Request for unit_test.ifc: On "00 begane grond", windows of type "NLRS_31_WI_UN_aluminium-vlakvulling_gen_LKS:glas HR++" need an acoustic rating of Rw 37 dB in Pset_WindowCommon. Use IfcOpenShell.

First a look at what the model holds.

```python
import ifcopenshell
import ifcopenshell.util.element

model = ifcopenshell.open("unit_test.ifc")
print(model.schema)
storey = next(s for s in model.by_type("IfcBuildingStorey") if s.Name == "00 begane grond")
windows = [e for e in ifcopenshell.util.element.get_decomposition(storey) if e.is_a("IfcWindow")]
seen = {}
for e in windows:
    element_type = ifcopenshell.util.element.get_type(e)
    key = (element_type.Name if element_type != e and element_type else None, ifcopenshell.util.element.get_pset(e, "Pset_WindowCommon", "AcousticRating"))
    seen[key] = seen.get(key, 0) + 1
for (name, value), count in sorted(seen.items(), key=str):
    print(count, "x", name, "|", value)
```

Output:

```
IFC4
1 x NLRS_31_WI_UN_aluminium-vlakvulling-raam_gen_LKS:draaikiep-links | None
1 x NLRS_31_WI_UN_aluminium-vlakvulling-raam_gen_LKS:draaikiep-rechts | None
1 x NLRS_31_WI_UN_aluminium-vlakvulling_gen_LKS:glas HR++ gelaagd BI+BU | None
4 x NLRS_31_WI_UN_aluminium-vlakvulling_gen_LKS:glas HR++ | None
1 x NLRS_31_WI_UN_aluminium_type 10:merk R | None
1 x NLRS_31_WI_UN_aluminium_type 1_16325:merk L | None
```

```python
import ifcopenshell
import ifcopenshell.api.pset
import ifcopenshell.util.element

model = ifcopenshell.open("unit_test.ifc")

storey = next(s for s in model.by_type("IfcBuildingStorey") if s.Name == "00 begane grond")
windows = [e for e in ifcopenshell.util.element.get_decomposition(storey) if e.is_a("IfcWindow")]

count = 0
for e in windows:
    element_type = ifcopenshell.util.element.get_type(e)
    if element_type in (None, e) or element_type.Name != "NLRS_31_WI_UN_aluminium-vlakvulling_gen_LKS:glas HR++":
        continue
    # add_pset returns the element's existing set when there is one.
    pset = ifcopenshell.api.pset.add_pset(model, product=e, name="Pset_WindowCommon")
    ifcopenshell.api.pset.edit_pset(model, pset=pset, properties={"AcousticRating": "Rw 37 dB"})
    count += 1

print(count, "windows updated")

model.write("unit_test-out.ifc")
```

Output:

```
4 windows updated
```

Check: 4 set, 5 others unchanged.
